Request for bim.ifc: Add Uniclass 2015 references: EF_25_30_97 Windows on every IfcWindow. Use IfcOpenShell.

First a look at what the model holds.

```python
import ifcopenshell

model = ifcopenshell.open("bim.ifc")
print(model.schema)
print("classifications:", [c.Name for c in model.by_type("IfcClassification")])
for ifc_class in ("IfcDoor", "IfcRoof", "IfcStair", "IfcWall", "IfcWindow"):
    print(ifc_class, len(model.by_type(ifc_class)))
```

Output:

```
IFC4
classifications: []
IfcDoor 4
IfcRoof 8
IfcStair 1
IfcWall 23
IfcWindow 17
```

```python
import ifcopenshell
import ifcopenshell.api.classification

model = ifcopenshell.open("bim.ifc")

system = ifcopenshell.api.classification.add_classification(model, classification="Uniclass 2015")

codes = {
    "IfcWindow": ("EF_25_30_97", "Windows"),
}
for ifc_class, (code, name) in codes.items():
    products = model.by_type(ifc_class)
    ifcopenshell.api.classification.add_reference(
        model, products=products, classification=system, identification=code, name=name
    )
    print(code, len(products))

model.write("bim-out.ifc")
```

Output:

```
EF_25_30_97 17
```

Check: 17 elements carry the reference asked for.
